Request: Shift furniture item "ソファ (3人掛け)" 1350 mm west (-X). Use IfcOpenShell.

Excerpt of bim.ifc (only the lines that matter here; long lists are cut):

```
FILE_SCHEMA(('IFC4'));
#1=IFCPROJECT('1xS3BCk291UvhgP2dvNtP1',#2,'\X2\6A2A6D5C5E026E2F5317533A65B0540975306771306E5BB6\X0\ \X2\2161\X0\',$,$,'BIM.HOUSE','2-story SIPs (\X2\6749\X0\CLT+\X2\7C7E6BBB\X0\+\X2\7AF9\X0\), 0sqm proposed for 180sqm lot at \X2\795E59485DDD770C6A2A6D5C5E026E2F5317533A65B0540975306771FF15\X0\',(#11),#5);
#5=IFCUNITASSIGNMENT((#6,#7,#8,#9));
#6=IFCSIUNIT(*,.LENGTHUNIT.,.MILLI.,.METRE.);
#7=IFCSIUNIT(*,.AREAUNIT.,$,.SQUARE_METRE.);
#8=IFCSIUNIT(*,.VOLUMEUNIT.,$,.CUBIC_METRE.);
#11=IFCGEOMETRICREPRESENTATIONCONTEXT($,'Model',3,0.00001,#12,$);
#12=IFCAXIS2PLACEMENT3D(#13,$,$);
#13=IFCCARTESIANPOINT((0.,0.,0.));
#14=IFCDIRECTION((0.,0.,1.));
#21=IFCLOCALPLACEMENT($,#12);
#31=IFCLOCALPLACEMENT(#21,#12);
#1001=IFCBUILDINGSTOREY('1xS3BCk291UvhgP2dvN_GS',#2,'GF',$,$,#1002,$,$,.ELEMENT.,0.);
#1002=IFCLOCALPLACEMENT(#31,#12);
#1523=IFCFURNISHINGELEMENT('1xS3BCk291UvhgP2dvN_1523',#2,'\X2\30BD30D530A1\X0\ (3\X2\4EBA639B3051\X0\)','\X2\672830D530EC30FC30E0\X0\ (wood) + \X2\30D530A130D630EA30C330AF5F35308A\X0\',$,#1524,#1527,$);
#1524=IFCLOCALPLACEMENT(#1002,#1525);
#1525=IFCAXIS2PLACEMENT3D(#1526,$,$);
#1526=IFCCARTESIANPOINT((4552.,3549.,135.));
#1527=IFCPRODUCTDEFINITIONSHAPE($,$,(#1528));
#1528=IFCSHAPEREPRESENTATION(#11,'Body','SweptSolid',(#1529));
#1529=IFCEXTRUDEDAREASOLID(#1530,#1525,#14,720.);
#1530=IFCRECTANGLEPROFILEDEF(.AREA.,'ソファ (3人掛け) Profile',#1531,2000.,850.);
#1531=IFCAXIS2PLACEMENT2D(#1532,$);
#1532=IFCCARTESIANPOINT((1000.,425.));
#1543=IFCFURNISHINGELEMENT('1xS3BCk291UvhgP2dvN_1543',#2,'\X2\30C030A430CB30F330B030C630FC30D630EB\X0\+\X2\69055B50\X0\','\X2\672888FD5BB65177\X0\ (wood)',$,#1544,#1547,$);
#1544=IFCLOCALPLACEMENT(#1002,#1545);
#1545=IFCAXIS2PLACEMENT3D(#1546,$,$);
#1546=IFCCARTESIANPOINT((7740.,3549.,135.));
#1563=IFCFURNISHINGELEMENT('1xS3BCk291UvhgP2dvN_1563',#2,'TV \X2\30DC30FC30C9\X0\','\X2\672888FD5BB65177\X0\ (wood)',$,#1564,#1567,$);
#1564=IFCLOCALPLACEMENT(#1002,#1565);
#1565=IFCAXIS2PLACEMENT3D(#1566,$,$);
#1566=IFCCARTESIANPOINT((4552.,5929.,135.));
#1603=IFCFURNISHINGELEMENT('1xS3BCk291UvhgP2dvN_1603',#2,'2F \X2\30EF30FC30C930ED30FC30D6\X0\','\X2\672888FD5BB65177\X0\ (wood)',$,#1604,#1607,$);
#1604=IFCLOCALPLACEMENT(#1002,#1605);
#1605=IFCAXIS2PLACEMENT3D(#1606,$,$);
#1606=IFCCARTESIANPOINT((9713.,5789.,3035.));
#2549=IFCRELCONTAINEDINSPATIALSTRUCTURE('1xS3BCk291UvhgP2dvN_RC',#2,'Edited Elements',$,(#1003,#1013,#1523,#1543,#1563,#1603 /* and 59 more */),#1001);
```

```python
import ifcopenshell
import ifcopenshell.api.geometry
import ifcopenshell.util.placement
import ifcopenshell.util.unit

model = ifcopenshell.open("bim.ifc")
unit_scale = ifcopenshell.util.unit.calculate_unit_scale(model)

item = model.by_guid("1xS3BCk291UvhgP2dvN_1523")
matrix = ifcopenshell.util.placement.get_local_placement(item.ObjectPlacement)
matrix[0, 3] -= 1.35 / unit_scale
ifcopenshell.api.geometry.edit_object_placement(model, product=item, matrix=matrix, is_si=False)

print(ifcopenshell.util.placement.get_local_placement(item.ObjectPlacement).round(3) + 0.0)

model.write("bim_rev.ifc")
```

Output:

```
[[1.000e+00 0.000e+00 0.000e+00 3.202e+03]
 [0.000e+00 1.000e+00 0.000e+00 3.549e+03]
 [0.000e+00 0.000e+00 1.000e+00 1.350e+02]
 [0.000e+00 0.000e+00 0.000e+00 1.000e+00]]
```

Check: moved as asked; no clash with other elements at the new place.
